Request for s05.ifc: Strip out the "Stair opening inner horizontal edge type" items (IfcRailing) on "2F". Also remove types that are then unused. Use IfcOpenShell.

First a look at what the model holds.

```python
import ifcopenshell
import ifcopenshell.util.element

model = ifcopenshell.open("s05.ifc")
print(model.schema)
storey = next(s for s in model.by_type("IfcBuildingStorey") if s.Name == "2F")
railings = [e for e in ifcopenshell.util.element.get_decomposition(storey) if e.is_a("IfcRailing")]
seen = {}
for e in railings:
    element_type = ifcopenshell.util.element.get_type(e)
    name = element_type.Name if element_type not in (None, e) else None
    seen[name] = seen.get(name, 0) + 1
for name, count in sorted(seen.items(), key=str):
    print(count, "x", name)
```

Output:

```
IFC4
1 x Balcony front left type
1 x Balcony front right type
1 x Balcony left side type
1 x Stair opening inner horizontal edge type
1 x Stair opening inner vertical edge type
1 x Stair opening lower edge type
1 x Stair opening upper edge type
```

```python
import ifcopenshell
import ifcopenshell.api.root
import ifcopenshell.util.element

model = ifcopenshell.open("s05.ifc")

storey = next(s for s in model.by_type("IfcBuildingStorey") if s.Name == "2F")
railings = [e for e in ifcopenshell.util.element.get_decomposition(storey) if e.is_a("IfcRailing")]
targets = [e for e in railings if (t := ifcopenshell.util.element.get_type(e)) not in (None, e) and t.Name == "Stair opening inner horizontal edge type"]
types = {ifcopenshell.util.element.get_type(e) for e in targets} - {None, *targets}

for e in targets:
    ifcopenshell.api.root.remove_product(model, product=e)
print(len(targets), "removed")

unused = [t for t in types if not ifcopenshell.util.element.get_types(t)]
for t in unused:
    ifcopenshell.api.root.remove_product(model, product=t)
print(len(unused), "unused types removed")

model.write("s05_updated.ifc")
```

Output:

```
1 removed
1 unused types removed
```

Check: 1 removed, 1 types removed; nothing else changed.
